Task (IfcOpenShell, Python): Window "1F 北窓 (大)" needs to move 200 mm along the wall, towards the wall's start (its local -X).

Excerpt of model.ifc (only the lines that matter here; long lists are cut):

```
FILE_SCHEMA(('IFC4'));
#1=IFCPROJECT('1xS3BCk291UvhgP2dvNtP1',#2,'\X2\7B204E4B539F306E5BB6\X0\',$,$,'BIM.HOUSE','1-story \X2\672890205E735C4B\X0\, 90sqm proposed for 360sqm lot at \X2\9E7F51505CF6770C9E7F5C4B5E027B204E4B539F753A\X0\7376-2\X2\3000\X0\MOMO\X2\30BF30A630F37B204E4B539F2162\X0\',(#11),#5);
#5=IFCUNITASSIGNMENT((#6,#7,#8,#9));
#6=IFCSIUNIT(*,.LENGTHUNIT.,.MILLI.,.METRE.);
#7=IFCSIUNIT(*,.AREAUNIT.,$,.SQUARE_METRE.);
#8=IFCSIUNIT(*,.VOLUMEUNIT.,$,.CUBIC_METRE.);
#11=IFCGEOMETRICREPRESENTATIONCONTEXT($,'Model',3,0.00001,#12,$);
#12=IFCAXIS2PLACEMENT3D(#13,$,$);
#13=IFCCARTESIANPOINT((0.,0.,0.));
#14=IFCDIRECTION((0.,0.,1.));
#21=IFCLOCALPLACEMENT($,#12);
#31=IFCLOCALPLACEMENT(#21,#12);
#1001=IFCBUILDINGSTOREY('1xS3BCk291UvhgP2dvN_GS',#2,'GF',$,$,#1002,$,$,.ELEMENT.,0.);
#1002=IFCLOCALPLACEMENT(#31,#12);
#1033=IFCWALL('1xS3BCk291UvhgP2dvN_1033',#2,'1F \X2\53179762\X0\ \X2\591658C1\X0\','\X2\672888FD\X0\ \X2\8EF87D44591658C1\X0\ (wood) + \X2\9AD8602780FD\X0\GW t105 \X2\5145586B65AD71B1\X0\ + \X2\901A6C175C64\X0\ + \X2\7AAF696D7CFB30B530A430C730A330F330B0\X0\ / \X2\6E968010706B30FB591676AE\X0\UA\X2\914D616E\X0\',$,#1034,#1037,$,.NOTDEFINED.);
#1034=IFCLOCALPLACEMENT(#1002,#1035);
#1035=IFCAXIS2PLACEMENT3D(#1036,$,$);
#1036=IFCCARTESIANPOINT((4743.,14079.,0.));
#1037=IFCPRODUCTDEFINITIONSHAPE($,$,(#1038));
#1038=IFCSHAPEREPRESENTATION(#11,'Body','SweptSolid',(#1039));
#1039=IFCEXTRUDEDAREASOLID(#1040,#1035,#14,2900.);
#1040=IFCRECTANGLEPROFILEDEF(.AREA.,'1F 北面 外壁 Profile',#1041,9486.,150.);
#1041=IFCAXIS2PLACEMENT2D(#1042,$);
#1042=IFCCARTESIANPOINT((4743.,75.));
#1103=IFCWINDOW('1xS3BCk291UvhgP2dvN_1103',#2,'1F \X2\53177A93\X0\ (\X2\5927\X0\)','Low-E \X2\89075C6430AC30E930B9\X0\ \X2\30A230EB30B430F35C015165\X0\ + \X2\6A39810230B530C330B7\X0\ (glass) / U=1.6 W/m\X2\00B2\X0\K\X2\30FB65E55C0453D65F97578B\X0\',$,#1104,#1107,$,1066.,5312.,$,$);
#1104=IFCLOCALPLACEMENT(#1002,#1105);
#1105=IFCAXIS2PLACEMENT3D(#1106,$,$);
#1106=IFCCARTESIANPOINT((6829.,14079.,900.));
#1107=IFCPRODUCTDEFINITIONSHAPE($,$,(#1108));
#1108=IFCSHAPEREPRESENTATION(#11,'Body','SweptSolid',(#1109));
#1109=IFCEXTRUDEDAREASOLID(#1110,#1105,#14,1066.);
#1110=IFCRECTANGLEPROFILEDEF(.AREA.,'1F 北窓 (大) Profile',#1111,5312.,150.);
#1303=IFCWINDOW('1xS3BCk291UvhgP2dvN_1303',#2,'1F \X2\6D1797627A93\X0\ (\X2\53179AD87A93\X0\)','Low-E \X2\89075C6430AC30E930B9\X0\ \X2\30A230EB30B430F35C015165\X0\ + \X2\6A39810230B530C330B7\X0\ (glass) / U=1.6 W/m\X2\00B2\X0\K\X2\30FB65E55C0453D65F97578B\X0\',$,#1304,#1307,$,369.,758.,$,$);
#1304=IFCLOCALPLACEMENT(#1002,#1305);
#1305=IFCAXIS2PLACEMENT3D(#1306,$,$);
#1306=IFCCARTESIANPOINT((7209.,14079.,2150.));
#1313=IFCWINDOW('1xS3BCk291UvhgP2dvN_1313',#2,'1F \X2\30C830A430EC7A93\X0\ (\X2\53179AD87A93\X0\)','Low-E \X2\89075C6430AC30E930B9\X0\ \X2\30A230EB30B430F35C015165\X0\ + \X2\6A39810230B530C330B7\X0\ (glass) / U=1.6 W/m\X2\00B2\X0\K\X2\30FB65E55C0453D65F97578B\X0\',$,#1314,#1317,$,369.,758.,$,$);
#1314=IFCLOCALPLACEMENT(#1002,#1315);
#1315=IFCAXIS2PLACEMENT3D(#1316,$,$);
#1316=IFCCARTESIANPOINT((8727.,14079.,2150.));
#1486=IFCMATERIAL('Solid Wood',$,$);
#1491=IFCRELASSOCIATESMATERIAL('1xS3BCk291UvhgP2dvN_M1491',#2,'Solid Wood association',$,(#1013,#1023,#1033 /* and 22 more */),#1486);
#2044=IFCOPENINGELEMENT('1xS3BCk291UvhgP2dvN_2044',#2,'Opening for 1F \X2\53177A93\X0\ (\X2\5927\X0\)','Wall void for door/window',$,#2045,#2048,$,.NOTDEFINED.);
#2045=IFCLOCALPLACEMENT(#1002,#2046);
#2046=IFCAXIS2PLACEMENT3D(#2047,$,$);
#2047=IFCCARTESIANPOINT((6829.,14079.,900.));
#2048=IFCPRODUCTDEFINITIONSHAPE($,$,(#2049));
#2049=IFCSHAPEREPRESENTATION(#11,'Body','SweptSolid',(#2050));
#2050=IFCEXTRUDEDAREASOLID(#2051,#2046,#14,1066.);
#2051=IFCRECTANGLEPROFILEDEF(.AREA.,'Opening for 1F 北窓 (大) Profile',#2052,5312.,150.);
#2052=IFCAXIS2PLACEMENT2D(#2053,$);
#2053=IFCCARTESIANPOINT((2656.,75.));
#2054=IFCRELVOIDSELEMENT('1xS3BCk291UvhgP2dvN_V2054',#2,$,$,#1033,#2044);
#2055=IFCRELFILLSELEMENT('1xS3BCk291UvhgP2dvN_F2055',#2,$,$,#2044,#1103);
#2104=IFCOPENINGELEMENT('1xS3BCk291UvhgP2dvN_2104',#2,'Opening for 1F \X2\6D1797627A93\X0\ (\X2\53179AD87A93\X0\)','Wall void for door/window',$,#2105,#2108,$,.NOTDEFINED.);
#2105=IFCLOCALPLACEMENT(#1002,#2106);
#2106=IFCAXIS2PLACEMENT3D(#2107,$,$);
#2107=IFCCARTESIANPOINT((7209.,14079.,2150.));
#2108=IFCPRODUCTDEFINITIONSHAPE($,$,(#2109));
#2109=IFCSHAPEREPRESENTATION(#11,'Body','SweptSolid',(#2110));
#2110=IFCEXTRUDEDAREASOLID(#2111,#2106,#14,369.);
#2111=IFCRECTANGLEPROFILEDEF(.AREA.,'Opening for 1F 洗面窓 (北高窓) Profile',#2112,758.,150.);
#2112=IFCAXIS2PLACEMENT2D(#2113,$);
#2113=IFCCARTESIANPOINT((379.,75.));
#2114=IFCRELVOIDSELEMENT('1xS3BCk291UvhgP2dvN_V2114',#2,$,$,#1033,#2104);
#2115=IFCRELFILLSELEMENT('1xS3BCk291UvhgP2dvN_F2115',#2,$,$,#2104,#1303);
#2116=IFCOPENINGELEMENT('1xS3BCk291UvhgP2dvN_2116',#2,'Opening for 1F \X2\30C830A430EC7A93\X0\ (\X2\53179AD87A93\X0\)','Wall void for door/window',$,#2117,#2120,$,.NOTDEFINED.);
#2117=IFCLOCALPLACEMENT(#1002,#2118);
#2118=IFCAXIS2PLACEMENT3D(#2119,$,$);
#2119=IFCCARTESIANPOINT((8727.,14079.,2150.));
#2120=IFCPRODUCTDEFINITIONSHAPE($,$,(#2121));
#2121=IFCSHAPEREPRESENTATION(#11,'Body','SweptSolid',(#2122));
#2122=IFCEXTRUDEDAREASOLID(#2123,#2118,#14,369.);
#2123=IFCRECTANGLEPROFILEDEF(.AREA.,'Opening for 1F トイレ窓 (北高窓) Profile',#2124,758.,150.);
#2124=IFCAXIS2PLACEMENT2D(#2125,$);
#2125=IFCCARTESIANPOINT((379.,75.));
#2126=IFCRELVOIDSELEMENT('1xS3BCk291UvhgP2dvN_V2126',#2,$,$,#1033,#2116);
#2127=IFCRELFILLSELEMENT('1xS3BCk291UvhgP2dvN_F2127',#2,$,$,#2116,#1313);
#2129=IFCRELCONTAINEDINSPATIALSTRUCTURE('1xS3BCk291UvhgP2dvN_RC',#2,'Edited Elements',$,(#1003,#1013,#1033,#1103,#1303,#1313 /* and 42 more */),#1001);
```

```python
import ifcopenshell
import ifcopenshell.api.geometry
import ifcopenshell.util.placement
import ifcopenshell.util.unit

model = ifcopenshell.open("model.ifc")
unit_scale = ifcopenshell.util.unit.calculate_unit_scale(model)

window = model.by_id(1103)
opening = window.FillsVoids[0].RelatingOpeningElement
wall = opening.VoidsElements[0].RelatingBuildingElement

wall_matrix = ifcopenshell.util.placement.get_local_placement(wall.ObjectPlacement)
shift = wall_matrix[:3, 0] * -0.2 / unit_scale
before = ifcopenshell.util.placement.get_local_placement(window.ObjectPlacement)[:3, 3].copy()

# The window is not placed relative to its opening, so move both.
for product in (opening, window):
    matrix = ifcopenshell.util.placement.get_local_placement(product.ObjectPlacement)
    matrix[:3, 3] += shift
    ifcopenshell.api.geometry.edit_object_placement(model, product=product, matrix=matrix, is_si=False)

after = ifcopenshell.util.placement.get_local_placement(window.ObjectPlacement)[:3, 3]
print("window moved by", (after - before).round(3) + 0.0)

model.write("model_v2.ifc")
```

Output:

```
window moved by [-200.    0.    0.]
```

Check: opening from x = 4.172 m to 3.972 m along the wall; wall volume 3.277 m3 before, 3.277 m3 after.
